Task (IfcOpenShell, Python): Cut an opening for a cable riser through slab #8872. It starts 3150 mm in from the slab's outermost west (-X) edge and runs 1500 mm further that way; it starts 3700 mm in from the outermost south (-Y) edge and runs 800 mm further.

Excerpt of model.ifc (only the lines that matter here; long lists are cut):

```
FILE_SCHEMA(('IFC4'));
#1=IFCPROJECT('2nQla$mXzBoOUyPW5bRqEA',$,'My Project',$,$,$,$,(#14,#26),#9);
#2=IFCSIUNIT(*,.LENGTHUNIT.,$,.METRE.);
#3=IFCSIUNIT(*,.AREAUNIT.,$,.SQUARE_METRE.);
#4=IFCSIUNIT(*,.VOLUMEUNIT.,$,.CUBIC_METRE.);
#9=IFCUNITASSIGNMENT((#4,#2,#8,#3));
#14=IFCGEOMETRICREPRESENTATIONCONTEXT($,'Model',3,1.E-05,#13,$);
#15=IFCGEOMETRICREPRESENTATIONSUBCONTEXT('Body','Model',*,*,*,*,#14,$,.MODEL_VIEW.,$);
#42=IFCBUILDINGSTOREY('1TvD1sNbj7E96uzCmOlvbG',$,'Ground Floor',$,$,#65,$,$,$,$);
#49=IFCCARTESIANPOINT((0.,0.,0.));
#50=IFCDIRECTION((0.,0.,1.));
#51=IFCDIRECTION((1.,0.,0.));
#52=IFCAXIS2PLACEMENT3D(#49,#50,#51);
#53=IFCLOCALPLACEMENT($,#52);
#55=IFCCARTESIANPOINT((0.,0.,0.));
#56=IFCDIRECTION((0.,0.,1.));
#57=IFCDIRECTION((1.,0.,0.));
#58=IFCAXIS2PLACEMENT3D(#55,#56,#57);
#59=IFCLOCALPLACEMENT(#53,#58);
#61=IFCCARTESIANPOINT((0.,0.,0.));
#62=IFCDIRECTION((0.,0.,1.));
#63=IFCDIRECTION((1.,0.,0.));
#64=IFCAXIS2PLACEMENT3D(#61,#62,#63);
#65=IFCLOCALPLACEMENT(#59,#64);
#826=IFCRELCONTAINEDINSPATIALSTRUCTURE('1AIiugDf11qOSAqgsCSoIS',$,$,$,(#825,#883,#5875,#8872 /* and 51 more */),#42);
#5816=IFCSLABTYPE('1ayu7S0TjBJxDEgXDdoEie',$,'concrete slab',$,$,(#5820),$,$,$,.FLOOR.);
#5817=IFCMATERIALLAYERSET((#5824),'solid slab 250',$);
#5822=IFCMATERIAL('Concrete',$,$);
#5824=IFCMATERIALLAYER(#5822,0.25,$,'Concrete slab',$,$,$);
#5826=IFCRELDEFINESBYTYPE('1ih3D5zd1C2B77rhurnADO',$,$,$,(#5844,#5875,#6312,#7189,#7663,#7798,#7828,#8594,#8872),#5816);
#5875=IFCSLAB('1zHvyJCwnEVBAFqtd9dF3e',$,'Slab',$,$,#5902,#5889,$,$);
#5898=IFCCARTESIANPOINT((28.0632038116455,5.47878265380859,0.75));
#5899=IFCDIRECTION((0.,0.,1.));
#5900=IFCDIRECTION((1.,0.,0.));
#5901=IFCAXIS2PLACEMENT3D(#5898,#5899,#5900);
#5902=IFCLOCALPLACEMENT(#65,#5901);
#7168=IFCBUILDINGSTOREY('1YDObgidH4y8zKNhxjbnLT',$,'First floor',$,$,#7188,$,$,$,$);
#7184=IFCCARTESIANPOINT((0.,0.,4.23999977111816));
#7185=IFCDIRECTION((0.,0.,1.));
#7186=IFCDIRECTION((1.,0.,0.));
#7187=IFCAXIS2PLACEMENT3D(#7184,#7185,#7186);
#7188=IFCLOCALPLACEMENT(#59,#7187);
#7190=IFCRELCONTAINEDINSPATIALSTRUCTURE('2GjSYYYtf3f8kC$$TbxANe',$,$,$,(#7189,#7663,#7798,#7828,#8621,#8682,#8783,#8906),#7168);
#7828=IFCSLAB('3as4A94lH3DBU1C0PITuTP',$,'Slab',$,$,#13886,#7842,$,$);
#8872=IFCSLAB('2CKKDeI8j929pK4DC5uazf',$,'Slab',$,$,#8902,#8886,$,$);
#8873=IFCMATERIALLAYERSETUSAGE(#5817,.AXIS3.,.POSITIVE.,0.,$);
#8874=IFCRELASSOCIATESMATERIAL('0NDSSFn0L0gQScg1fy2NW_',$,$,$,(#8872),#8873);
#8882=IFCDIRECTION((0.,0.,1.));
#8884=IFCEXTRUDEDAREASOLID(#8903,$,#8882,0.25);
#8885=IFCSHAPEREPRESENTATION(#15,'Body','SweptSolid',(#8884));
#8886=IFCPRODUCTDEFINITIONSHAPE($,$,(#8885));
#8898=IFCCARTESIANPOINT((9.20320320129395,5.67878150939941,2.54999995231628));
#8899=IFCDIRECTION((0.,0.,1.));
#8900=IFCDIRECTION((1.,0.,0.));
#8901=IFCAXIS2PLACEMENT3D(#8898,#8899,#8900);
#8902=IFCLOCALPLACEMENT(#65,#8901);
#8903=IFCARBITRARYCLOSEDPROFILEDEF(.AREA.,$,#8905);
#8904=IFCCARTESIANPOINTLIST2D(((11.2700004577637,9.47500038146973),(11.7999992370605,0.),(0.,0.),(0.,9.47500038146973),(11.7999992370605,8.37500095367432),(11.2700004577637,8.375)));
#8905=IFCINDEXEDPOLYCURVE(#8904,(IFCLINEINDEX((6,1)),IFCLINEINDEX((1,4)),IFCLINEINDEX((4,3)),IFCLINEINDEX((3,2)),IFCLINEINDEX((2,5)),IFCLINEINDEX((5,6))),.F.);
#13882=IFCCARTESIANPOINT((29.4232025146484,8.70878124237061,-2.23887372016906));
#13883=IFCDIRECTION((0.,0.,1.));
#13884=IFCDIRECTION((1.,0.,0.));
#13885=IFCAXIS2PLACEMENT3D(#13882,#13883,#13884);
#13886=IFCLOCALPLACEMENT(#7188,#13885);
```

```python
import numpy as np
import ifcopenshell
import ifcopenshell.api.feature
import ifcopenshell.api.geometry
import ifcopenshell.api.root
import ifcopenshell.geom
import ifcopenshell.util.placement
import ifcopenshell.util.representation
import ifcopenshell.util.shape
import ifcopenshell.util.unit

model = ifcopenshell.open("model.ifc")
unit_scale = ifcopenshell.util.unit.calculate_unit_scale(model)
settings = ifcopenshell.geom.settings()


def volume(element):
    """Net volume in cubic metres, openings subtracted."""
    shape = ifcopenshell.geom.create_shape(settings, element)
    return ifcopenshell.util.shape.get_volume(shape.geometry)


slab = model.by_guid("2CKKDeI8j929pK4DC5uazf")
before = volume(slab)

# Extent in the slab's own axes, in metres. The edges named are its -X and -Y sides.
slab_shape = ifcopenshell.geom.create_shape(settings, slab)
vertices = ifcopenshell.util.shape.get_vertices(slab_shape.geometry)
x_min, y_min, bottom = vertices.min(axis=0)
top = vertices[:, 2].max()

opening = ifcopenshell.api.root.create_entity(model, ifc_class="IfcOpeningElement", name="Cable riser opening", predefined_type="OPENING")
context = ifcopenshell.util.representation.get_context(model, "Model", "Body", "MODEL_VIEW")
width, depth = 1.5, 0.8
outline = [(0.0, 0.0), (width, 0.0), (width, depth), (0.0, depth), (0.0, 0.0)]
# Overshoot both faces by 50 mm so the cut is clean.
shape = ifcopenshell.api.geometry.add_slab_representation(
    model, context=context, depth=top - bottom + 0.1, polyline=outline
)
ifcopenshell.api.geometry.assign_representation(model, product=opening, representation=shape)

matrix = ifcopenshell.util.placement.get_local_placement(slab.ObjectPlacement)
matrix[:, 3] = matrix @ np.append(np.array([x_min + 3.15, y_min + 3.7, bottom - 0.05]) / unit_scale, 1.0)
ifcopenshell.api.geometry.edit_object_placement(model, product=opening, matrix=matrix, is_si=False)
ifcopenshell.api.feature.add_feature(model, feature=opening, element=slab)

after = volume(slab)

print(f"slab volume {before:.3f} -> {after:.3f} m3")

model.write("model_edited.ifc")
```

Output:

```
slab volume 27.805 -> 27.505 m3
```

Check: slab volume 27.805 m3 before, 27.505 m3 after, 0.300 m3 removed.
